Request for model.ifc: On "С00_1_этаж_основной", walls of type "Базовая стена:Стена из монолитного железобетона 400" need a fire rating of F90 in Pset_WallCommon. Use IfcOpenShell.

First a look at what the model holds.

```python
import ifcopenshell
import ifcopenshell.util.element

model = ifcopenshell.open("model.ifc")
print(model.schema)
storey = next(s for s in model.by_type("IfcBuildingStorey") if s.Name == "С00_1_этаж_основной")
walls = [e for e in ifcopenshell.util.element.get_decomposition(storey) if e.is_a("IfcWall")]
seen = {}
for e in walls:
    element_type = ifcopenshell.util.element.get_type(e)
    key = (element_type.Name if element_type != e and element_type else None, ifcopenshell.util.element.get_pset(e, "Pset_WallCommon", "FireRating"))
    seen[key] = seen.get(key, 0) + 1
for (name, value), count in sorted(seen.items(), key=str):
    print(count, "x", name, "|", value)
```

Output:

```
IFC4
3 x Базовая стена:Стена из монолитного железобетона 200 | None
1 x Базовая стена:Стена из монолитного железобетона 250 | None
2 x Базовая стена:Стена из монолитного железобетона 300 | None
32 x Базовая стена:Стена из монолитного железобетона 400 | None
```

```python
import ifcopenshell
import ifcopenshell.api.pset
import ifcopenshell.util.element

model = ifcopenshell.open("model.ifc")

storey = next(s for s in model.by_type("IfcBuildingStorey") if s.Name == "С00_1_этаж_основной")
walls = [e for e in ifcopenshell.util.element.get_decomposition(storey) if e.is_a("IfcWall")]

count = 0
for e in walls:
    element_type = ifcopenshell.util.element.get_type(e)
    if element_type in (None, e) or element_type.Name != "Базовая стена:Стена из монолитного железобетона 400":
        continue
    # add_pset returns the element's existing set when there is one.
    pset = ifcopenshell.api.pset.add_pset(model, product=e, name="Pset_WallCommon")
    ifcopenshell.api.pset.edit_pset(model, pset=pset, properties={"FireRating": "F90"})
    count += 1

print(count, "walls updated")

model.write("model_updated.ifc")
```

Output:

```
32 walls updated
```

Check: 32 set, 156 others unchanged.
